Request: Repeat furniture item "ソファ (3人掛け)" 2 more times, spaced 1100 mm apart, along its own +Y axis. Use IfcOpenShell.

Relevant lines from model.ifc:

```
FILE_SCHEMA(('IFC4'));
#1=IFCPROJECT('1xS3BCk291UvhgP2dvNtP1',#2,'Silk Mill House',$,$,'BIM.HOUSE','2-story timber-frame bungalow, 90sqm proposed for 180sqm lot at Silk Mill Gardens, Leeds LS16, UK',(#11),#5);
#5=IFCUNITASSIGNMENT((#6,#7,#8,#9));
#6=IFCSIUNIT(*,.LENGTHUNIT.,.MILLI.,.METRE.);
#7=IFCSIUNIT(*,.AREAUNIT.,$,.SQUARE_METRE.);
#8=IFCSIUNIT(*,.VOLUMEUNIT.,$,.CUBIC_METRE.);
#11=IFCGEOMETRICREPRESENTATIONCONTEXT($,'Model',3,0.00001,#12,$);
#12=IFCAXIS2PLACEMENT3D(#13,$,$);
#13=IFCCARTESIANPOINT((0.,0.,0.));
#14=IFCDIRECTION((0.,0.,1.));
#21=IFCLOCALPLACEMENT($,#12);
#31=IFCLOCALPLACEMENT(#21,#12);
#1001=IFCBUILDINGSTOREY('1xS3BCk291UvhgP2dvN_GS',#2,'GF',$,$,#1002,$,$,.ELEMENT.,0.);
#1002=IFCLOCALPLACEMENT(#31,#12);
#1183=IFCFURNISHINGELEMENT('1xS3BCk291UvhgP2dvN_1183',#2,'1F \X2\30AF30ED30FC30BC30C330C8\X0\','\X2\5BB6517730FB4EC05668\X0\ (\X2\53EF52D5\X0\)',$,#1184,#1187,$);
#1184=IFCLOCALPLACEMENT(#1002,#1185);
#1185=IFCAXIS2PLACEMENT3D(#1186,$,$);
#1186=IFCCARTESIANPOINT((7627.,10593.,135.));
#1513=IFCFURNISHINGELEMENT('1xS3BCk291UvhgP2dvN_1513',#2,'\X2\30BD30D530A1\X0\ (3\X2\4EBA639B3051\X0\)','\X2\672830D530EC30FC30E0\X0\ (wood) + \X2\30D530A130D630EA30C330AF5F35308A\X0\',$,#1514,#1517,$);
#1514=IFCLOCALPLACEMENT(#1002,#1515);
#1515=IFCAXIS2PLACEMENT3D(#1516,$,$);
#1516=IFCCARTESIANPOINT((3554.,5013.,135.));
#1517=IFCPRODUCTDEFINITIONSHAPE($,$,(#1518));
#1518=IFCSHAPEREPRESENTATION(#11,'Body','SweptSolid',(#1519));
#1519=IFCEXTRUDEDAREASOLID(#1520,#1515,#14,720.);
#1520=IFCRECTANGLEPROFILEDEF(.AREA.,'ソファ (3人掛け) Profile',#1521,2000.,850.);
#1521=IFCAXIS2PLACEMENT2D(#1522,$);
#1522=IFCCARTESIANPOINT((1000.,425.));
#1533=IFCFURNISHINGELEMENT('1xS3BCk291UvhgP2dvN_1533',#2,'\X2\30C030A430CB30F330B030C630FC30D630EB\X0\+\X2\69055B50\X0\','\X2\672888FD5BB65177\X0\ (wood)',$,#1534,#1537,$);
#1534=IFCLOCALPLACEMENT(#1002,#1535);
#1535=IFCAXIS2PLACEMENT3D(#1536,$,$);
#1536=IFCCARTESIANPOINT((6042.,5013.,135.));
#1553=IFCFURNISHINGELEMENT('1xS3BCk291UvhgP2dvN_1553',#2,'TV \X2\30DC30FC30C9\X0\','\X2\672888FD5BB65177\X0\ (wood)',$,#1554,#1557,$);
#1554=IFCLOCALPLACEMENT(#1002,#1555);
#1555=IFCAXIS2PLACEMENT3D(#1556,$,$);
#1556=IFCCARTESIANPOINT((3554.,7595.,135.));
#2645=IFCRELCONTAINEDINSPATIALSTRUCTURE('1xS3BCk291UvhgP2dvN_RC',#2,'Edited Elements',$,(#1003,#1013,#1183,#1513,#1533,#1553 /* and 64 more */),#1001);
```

```python
import ifcopenshell
import ifcopenshell.api.geometry
import ifcopenshell.api.root
import ifcopenshell.util.element
import ifcopenshell.util.placement

model = ifcopenshell.open("model.ifc")


def reuse_history(source, copy):
    """copy_class also copies each property set's owner history, people and application; keep the originals."""
    for rel in copy.IsDefinedBy:
        if rel.is_a("IfcRelDefinesByProperties") and (history := rel.RelatingPropertyDefinition.OwnerHistory):
            rel.RelatingPropertyDefinition.OwnerHistory = source.OwnerHistory
            ifcopenshell.util.element.remove_deep2(model, history)


source = model.by_guid("1xS3BCk291UvhgP2dvN_1513")
base = ifcopenshell.util.placement.get_local_placement(source.ObjectPlacement)
step = base[:3, 1] * 1100.0

for i in range(1, 3):
    copy = ifcopenshell.api.root.copy_class(model, product=source)
    copy.Representation = ifcopenshell.util.element.copy_deep(
        model, source.Representation, exclude=["IfcGeometricRepresentationContext", "IfcRepresentationMap"]
    )
    reuse_history(source, copy)
    matrix = base.copy()
    matrix[:3, 3] += i * step
    print("added at", matrix[:3, 3].round(3) + 0.0)
    ifcopenshell.api.geometry.edit_object_placement(model, product=copy, matrix=matrix, is_si=False)

model.write("model_updated.ifc")
```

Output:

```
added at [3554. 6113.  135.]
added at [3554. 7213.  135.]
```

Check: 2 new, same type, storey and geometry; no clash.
